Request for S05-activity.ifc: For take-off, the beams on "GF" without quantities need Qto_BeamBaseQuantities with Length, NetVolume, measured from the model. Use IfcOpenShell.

First a look at what the model holds.

```python
import ifcopenshell
import ifcopenshell.util.element
import ifcopenshell.util.unit

model = ifcopenshell.open("S05-activity.ifc")
print(model.schema)
for unit_type in ("LENGTHUNIT", "AREAUNIT", "VOLUMEUNIT"):
    print(unit_type, ifcopenshell.util.unit.calculate_unit_scale(model, unit_type))
storey = next(s for s in model.by_type("IfcBuildingStorey") if s.Name == "GF")
beams = [e for e in ifcopenshell.util.element.get_decomposition(storey) if e.is_a("IfcBeam")]
for e in sorted(beams, key=lambda e: e.id()):
    print(e.id(), e.is_a(), e.Name, list(ifcopenshell.util.element.get_psets(e, qtos_only=True)), sep=" | ")
```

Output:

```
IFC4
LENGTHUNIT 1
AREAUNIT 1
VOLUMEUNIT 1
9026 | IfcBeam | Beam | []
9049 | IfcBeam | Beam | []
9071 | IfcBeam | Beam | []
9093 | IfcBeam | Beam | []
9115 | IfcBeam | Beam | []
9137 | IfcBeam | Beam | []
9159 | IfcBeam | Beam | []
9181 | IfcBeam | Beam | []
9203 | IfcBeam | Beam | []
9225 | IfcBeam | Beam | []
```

```python
import ifcopenshell
import ifcopenshell.api.pset
import ifcopenshell.geom
import ifcopenshell.util.element
import ifcopenshell.util.shape
import ifcopenshell.util.unit

model = ifcopenshell.open("S05-activity.ifc")
unit_scale = ifcopenshell.util.unit.calculate_unit_scale(model)
volume_scale = ifcopenshell.util.unit.calculate_unit_scale(model, "VOLUMEUNIT")
settings = ifcopenshell.geom.settings()

storey = next(s for s in model.by_type("IfcBuildingStorey") if s.Name == "GF")
beams = [e for e in ifcopenshell.util.element.get_decomposition(storey) if e.is_a("IfcBeam")]

for e in sorted(beams, key=lambda e: e.id()):
    if ifcopenshell.util.element.get_psets(e, qtos_only=True, should_inherit=False):
        continue
    # Geometry comes back in metres, in the element's own axes.
    shape = ifcopenshell.geom.create_shape(settings, e)
    values = {
        "Length": ifcopenshell.util.shape.get_max_xyz(shape.geometry) / unit_scale,
        "NetVolume": ifcopenshell.util.shape.get_volume(shape.geometry) / volume_scale,
    }
    qto = ifcopenshell.api.pset.add_qto(model, product=e, name="Qto_BeamBaseQuantities")
    ifcopenshell.api.pset.edit_qto(model, qto=qto, properties=values)
    print(e.id(), {k: round(v, 3) for k, v in values.items()})

model.write("S05-activity_rev.ifc")
```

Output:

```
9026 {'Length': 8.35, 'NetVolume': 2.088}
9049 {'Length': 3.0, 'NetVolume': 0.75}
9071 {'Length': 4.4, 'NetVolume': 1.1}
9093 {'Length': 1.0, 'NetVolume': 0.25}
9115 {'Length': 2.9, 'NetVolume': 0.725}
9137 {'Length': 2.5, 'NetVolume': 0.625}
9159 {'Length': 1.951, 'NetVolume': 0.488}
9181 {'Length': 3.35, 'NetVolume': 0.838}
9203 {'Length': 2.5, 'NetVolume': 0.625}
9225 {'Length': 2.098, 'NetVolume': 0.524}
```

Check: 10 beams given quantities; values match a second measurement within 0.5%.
